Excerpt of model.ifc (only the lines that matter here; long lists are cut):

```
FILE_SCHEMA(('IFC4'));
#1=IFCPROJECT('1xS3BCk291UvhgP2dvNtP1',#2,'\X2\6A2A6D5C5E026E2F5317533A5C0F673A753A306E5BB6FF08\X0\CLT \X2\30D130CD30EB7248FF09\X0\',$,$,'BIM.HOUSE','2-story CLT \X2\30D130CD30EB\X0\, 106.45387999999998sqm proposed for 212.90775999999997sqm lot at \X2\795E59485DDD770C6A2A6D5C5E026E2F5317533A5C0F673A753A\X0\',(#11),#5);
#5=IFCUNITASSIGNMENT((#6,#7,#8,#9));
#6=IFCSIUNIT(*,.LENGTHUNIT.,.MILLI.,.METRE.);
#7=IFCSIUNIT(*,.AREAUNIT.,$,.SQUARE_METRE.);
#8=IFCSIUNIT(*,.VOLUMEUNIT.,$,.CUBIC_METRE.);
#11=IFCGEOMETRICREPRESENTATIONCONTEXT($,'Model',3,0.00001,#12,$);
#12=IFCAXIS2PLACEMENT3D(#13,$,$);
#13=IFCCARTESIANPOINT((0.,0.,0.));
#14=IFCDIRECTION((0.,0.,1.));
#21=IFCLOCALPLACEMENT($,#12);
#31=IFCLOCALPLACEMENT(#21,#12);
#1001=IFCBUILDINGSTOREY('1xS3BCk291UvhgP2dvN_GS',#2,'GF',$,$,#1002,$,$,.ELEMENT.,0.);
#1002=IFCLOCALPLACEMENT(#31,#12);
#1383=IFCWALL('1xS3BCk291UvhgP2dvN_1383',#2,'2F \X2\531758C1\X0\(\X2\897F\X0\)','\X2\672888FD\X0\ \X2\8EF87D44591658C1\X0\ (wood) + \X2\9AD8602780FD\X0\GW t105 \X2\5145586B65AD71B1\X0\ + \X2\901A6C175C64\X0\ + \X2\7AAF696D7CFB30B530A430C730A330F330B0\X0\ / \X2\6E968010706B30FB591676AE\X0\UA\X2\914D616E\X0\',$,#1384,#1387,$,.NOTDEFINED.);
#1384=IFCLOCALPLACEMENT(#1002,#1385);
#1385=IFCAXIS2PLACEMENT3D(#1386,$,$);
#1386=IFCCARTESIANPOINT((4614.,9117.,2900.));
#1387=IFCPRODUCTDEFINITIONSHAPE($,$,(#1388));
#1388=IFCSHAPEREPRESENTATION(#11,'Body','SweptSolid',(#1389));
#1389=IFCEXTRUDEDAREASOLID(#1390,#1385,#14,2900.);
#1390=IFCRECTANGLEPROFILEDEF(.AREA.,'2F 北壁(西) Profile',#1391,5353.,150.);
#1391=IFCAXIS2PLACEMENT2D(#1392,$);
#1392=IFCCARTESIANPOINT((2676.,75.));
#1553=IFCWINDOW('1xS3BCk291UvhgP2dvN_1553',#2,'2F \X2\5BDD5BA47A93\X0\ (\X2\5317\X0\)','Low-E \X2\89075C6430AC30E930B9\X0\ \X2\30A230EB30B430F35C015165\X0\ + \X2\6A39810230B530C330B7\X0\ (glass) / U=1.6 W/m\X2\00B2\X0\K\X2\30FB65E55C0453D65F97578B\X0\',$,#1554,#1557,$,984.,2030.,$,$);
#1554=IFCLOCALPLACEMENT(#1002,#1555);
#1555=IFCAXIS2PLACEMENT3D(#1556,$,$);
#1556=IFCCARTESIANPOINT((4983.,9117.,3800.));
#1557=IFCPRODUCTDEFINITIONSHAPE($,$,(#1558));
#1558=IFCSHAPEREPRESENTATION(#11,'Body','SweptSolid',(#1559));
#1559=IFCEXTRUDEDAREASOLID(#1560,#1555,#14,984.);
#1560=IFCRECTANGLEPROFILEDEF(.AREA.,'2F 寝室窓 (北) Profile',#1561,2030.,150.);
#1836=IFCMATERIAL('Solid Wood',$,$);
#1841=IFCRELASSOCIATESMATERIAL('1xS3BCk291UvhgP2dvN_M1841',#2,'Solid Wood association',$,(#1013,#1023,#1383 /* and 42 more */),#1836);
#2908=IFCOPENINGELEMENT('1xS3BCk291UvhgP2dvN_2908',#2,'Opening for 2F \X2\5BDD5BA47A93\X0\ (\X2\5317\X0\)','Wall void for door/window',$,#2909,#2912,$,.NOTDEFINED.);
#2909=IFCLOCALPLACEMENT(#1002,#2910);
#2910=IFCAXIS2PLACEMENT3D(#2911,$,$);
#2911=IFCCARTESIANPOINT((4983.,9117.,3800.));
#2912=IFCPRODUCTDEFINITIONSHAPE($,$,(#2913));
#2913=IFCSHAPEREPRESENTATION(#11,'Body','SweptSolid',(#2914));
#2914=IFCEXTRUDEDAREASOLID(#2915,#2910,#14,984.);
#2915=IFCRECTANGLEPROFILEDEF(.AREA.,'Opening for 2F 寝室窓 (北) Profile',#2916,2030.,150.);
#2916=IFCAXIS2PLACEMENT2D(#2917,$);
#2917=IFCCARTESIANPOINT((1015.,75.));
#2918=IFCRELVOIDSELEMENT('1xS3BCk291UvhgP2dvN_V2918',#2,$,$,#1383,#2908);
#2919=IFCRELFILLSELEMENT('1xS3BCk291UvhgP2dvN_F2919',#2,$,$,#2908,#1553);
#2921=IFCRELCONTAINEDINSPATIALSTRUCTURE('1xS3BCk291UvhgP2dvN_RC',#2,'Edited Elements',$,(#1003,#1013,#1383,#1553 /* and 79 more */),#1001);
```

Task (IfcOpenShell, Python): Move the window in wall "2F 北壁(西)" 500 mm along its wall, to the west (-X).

```python
import ifcopenshell
import ifcopenshell.api.geometry
import ifcopenshell.util.placement
import ifcopenshell.util.unit

model = ifcopenshell.open("model.ifc")
unit_scale = ifcopenshell.util.unit.calculate_unit_scale(model)

window = model.by_guid("1xS3BCk291UvhgP2dvN_1553")
opening = window.FillsVoids[0].RelatingOpeningElement
wall = opening.VoidsElements[0].RelatingBuildingElement

wall_matrix = ifcopenshell.util.placement.get_local_placement(wall.ObjectPlacement)
shift = wall_matrix[:3, 0] * -0.5 / unit_scale
before = ifcopenshell.util.placement.get_local_placement(window.ObjectPlacement)[:3, 3].copy()

# The window is not placed relative to its opening, so move both.
for product in (opening, window):
    matrix = ifcopenshell.util.placement.get_local_placement(product.ObjectPlacement)
    matrix[:3, 3] += shift
    ifcopenshell.api.geometry.edit_object_placement(model, product=product, matrix=matrix, is_si=False)

after = ifcopenshell.util.placement.get_local_placement(window.ObjectPlacement)[:3, 3]
print("window moved by", (after - before).round(3) + 0.0)

model.write("model_v2.ifc")
```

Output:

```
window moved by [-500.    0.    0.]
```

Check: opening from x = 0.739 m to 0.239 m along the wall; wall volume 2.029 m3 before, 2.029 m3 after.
